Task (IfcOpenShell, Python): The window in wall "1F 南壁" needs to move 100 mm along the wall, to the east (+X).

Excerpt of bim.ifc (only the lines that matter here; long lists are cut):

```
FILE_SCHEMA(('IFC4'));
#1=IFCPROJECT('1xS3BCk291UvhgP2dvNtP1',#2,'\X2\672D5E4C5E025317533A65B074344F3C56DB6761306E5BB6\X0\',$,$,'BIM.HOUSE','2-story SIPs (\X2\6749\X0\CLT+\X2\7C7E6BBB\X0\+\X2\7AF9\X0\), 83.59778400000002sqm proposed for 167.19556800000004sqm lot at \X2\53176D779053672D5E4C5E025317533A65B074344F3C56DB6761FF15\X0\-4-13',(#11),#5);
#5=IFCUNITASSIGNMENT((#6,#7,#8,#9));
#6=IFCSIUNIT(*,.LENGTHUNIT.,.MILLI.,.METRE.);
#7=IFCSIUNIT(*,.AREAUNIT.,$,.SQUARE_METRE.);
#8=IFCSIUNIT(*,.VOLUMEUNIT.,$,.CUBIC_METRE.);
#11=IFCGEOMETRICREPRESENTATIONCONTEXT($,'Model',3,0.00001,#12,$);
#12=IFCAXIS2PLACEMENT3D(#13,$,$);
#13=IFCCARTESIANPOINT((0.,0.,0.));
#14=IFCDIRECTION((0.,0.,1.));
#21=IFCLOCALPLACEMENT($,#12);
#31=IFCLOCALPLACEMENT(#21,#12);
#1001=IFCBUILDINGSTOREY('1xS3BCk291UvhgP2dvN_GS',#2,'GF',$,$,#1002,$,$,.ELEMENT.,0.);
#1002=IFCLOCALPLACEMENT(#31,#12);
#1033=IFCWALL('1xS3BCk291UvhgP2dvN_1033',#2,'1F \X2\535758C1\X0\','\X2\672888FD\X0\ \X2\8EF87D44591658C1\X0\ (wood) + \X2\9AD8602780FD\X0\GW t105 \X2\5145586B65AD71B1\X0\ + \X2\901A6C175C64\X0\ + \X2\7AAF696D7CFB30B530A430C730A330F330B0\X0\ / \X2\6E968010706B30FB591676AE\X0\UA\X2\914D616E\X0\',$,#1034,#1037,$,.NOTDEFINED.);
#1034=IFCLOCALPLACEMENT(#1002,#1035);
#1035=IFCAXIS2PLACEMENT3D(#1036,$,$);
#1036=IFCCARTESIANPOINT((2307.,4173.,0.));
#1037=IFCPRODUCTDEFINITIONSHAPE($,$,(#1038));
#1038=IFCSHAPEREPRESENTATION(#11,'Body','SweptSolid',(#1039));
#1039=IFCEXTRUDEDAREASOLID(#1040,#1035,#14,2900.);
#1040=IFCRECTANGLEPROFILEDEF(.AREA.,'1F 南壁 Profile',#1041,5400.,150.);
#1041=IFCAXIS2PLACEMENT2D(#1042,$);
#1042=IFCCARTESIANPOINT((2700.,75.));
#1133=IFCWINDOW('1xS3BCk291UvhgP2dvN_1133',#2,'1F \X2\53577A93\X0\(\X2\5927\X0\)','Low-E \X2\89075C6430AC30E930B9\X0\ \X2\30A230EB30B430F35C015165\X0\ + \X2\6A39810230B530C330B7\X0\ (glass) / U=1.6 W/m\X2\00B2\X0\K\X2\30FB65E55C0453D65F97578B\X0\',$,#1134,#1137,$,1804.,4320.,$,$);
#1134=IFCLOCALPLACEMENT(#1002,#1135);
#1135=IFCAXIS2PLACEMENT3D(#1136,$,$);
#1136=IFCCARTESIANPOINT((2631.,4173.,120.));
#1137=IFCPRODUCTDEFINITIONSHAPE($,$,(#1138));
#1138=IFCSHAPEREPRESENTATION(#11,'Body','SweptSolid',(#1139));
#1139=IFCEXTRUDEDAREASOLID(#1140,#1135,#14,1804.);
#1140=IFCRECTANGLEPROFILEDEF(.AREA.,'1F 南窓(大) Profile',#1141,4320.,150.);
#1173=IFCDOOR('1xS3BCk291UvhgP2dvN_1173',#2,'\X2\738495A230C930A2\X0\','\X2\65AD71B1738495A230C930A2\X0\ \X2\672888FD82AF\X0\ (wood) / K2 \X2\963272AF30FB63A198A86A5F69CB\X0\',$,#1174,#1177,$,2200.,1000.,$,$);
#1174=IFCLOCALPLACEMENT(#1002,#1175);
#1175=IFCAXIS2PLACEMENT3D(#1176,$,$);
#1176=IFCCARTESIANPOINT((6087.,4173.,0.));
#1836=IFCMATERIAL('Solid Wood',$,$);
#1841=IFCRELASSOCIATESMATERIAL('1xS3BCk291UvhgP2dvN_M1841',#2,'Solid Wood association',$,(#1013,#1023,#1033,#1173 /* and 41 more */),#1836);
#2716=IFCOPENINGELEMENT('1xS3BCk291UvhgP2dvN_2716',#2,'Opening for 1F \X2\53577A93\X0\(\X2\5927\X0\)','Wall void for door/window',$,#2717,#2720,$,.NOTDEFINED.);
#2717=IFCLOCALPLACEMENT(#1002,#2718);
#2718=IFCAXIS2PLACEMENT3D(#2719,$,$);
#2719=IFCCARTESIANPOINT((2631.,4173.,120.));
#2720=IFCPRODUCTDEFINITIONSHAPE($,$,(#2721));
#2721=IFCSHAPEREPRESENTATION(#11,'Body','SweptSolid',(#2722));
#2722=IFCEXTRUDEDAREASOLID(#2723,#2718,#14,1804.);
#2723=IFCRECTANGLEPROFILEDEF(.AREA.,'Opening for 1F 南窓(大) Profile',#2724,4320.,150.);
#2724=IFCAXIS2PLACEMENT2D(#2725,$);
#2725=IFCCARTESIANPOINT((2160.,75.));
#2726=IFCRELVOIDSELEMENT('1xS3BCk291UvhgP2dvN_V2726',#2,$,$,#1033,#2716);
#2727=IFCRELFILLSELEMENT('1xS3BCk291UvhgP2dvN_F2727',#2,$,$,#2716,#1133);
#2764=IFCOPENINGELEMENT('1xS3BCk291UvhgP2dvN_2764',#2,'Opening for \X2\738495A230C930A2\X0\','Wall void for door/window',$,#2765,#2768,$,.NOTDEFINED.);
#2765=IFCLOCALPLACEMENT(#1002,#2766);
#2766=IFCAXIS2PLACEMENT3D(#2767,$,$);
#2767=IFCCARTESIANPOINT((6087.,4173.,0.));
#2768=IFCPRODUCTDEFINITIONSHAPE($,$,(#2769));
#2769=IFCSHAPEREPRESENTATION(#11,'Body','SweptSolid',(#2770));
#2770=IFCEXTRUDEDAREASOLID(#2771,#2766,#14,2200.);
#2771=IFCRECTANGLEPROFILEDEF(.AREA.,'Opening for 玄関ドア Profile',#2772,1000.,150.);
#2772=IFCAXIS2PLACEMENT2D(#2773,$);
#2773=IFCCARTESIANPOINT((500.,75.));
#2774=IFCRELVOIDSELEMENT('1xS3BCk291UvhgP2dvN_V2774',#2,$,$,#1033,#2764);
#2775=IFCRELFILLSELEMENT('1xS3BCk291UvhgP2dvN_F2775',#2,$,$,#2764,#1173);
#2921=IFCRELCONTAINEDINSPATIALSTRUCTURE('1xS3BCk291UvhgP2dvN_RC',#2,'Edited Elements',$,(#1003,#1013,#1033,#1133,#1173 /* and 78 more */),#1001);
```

```python
import ifcopenshell
import ifcopenshell.api.geometry
import ifcopenshell.util.placement
import ifcopenshell.util.unit

model = ifcopenshell.open("bim.ifc")
unit_scale = ifcopenshell.util.unit.calculate_unit_scale(model)

window = model.by_guid("1xS3BCk291UvhgP2dvN_1133")
opening = window.FillsVoids[0].RelatingOpeningElement
wall = opening.VoidsElements[0].RelatingBuildingElement

wall_matrix = ifcopenshell.util.placement.get_local_placement(wall.ObjectPlacement)
shift = wall_matrix[:3, 0] * 0.1 / unit_scale
before = ifcopenshell.util.placement.get_local_placement(window.ObjectPlacement)[:3, 3].copy()

# The window is not placed relative to its opening, so move both.
for product in (opening, window):
    matrix = ifcopenshell.util.placement.get_local_placement(product.ObjectPlacement)
    matrix[:3, 3] += shift
    ifcopenshell.api.geometry.edit_object_placement(model, product=product, matrix=matrix, is_si=False)

after = ifcopenshell.util.placement.get_local_placement(window.ObjectPlacement)[:3, 3]
print("window moved by", (after - before).round(3) + 0.0)

model.write("bim_updated.ifc")
```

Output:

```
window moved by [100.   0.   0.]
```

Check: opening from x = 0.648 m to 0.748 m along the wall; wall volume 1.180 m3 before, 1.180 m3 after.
